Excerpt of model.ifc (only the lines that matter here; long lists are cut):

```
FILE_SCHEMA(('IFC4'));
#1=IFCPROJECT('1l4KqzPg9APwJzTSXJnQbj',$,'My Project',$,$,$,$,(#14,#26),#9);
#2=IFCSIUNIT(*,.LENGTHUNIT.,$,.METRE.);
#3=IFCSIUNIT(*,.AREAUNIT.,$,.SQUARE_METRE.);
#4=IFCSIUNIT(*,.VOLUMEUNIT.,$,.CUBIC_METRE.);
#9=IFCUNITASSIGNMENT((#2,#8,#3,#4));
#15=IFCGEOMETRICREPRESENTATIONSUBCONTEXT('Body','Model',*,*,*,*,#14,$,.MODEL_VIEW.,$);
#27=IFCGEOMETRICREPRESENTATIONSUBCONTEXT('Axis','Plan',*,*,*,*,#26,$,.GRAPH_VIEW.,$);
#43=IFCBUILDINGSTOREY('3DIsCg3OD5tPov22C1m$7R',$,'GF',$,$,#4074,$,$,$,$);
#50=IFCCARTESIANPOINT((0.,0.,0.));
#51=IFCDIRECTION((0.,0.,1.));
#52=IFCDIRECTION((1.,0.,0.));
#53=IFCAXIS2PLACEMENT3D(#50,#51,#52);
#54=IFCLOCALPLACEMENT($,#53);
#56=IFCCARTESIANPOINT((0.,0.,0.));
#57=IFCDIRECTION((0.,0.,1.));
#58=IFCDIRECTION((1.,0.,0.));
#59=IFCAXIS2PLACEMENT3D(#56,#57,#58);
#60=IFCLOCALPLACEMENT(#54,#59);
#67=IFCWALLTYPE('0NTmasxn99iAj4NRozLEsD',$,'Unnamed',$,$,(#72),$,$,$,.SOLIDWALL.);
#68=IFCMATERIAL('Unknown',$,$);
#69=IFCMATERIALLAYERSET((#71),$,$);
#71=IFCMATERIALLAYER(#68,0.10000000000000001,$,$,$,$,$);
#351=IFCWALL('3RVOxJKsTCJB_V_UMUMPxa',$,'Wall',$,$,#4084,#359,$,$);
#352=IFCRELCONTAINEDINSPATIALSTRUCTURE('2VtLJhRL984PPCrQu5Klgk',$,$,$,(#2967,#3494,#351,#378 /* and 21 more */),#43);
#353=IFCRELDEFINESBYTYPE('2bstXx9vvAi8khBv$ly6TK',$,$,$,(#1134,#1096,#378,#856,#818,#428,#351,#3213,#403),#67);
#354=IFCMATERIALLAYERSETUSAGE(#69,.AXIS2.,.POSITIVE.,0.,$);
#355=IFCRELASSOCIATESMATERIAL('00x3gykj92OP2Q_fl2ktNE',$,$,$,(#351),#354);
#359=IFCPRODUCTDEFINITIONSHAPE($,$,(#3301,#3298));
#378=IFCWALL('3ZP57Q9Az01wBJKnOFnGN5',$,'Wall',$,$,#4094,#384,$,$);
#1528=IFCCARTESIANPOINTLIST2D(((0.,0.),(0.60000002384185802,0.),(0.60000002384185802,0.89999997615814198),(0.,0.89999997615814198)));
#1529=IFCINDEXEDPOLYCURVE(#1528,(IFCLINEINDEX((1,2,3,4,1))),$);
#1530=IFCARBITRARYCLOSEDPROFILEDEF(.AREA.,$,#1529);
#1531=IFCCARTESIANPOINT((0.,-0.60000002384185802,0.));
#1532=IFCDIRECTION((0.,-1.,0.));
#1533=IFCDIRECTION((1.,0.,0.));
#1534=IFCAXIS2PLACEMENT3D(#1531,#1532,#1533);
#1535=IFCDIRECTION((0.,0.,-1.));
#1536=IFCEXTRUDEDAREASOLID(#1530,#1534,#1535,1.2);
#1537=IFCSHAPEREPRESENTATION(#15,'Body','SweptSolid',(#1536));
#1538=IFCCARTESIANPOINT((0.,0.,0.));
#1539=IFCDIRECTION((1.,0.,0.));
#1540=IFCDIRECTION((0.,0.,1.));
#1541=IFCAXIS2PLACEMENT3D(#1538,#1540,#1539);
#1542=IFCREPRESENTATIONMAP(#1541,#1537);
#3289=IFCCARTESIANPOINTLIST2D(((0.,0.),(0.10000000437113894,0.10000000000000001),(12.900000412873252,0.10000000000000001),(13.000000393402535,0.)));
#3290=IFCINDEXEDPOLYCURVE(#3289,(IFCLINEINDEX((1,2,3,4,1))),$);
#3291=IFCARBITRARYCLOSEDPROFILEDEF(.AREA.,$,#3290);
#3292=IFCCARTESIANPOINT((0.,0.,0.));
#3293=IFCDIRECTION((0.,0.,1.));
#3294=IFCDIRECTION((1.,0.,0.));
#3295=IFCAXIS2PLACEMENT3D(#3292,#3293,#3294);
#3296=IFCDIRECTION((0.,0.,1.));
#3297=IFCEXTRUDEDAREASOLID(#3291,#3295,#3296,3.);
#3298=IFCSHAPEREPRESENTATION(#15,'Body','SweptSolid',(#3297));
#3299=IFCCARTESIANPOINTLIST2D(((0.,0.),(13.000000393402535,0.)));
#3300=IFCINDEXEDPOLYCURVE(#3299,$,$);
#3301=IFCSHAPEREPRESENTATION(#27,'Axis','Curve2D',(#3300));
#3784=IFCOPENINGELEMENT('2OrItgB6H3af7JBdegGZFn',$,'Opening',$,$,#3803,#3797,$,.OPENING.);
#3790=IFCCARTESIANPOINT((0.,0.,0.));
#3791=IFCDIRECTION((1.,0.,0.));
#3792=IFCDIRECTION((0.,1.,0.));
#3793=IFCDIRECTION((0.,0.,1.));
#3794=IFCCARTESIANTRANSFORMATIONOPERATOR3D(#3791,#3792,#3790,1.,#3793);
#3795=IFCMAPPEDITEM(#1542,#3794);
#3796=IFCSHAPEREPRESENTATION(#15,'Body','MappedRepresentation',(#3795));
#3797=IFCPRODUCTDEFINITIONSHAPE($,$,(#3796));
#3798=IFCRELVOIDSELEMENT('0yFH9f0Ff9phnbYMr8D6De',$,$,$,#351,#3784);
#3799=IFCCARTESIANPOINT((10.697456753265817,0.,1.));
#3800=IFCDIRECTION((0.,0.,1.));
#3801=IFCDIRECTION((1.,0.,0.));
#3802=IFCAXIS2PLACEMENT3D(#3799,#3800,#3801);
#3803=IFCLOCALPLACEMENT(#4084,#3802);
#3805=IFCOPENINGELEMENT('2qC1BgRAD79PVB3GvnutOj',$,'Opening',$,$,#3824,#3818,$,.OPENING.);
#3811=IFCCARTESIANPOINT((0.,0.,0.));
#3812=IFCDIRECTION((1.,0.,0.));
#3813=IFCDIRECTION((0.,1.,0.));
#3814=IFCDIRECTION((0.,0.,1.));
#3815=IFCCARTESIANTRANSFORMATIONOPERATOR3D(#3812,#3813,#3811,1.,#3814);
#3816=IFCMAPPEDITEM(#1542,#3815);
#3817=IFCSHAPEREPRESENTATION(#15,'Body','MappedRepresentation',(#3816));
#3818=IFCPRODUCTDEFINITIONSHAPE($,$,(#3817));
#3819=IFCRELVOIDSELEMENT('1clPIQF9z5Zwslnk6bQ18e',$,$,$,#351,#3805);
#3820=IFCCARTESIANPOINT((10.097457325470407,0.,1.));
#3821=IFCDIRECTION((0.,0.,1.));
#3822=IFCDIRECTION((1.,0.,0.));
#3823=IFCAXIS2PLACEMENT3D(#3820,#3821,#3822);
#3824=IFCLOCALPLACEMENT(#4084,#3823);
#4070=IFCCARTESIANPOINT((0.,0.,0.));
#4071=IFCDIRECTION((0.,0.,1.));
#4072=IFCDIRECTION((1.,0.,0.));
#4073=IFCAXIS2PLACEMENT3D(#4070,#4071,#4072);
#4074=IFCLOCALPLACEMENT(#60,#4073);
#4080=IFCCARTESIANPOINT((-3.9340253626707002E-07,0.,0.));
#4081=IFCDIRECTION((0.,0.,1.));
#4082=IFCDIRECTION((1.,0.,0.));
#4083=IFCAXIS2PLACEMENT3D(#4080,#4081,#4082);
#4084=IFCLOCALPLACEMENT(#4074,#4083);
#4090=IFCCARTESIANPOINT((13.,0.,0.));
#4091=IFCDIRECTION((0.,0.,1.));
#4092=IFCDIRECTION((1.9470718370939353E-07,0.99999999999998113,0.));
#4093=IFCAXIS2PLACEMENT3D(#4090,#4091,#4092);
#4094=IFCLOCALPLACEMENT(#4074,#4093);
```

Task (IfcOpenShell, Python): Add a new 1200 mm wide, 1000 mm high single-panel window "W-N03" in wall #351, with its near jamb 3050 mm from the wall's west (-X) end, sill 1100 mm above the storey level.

```python
import numpy as np
import ifcopenshell
import ifcopenshell.api.feature
import ifcopenshell.api.geometry
import ifcopenshell.api.root
import ifcopenshell.api.spatial
import ifcopenshell.geom
import ifcopenshell.util.element
import ifcopenshell.util.placement
import ifcopenshell.util.representation
import ifcopenshell.util.shape
import ifcopenshell.util.unit

model = ifcopenshell.open("model.ifc")
unit_scale = ifcopenshell.util.unit.calculate_unit_scale(model)
settings = ifcopenshell.geom.settings()


def volume(element):
    """Net volume in cubic metres, openings subtracted."""
    shape = ifcopenshell.geom.create_shape(settings, element)
    return ifcopenshell.util.shape.get_volume(shape.geometry)


wall = model.by_guid("3RVOxJKsTCJB_V_UMUMPxa")
storey = ifcopenshell.util.element.get_container(wall, ifc_class="IfcBuildingStorey")
context = ifcopenshell.util.representation.get_context(model, "Model", "Body", "MODEL_VIEW")
before = volume(wall)

width, height, from_end, sill = 1.2, 1, 3.05, 1.1  # metres

# The wall runs along its own X axis, and the end named is its -X end.
wall_shape = ifcopenshell.geom.create_shape(settings, wall)
x, y, z = ifcopenshell.util.shape.get_vertices(wall_shape.geometry).T
start = x.min() + from_end
face, thickness = float(y.min()), float(y.max() - y.min())
wall_matrix = ifcopenshell.util.placement.get_local_placement(wall.ObjectPlacement)
level = ifcopenshell.util.placement.get_local_placement(storey.ObjectPlacement)[2, 3]


def in_wall(x, y):
    """Placement at x, y metres in the wall's axes, at sill height."""
    matrix = wall_matrix.copy()
    matrix[:, 3] = wall_matrix @ np.array([x / unit_scale, y / unit_scale, 0.0, 1.0])
    matrix[2, 3] = level + sill / unit_scale
    return matrix


# Opening: a box that overshoots both wall faces by 50 mm.
opening = ifcopenshell.api.root.create_entity(model, ifc_class="IfcOpeningElement", predefined_type="OPENING")
box = ifcopenshell.api.geometry.add_wall_representation(
    model, context=context, length=width, height=height, thickness=thickness + 0.1
)
ifcopenshell.api.geometry.assign_representation(model, product=opening, representation=box)
ifcopenshell.api.geometry.edit_object_placement(model, product=opening, matrix=in_wall(start, face - 0.05), is_si=False)
ifcopenshell.api.feature.add_feature(model, feature=opening, element=wall)

window = ifcopenshell.api.root.create_entity(model, ifc_class="IfcWindow", name="W-N03", predefined_type="WINDOW")
window.OverallWidth, window.OverallHeight = width / unit_scale, height / unit_scale
window.PartitioningType = "SINGLE_PANEL"
body = ifcopenshell.api.geometry.add_window_representation(
    model,
    context=context,
    overall_width=window.OverallWidth,
    overall_height=window.OverallHeight,
    partition_type="SINGLE_PANEL",
)
ifcopenshell.api.geometry.assign_representation(model, product=window, representation=body)
ifcopenshell.api.spatial.assign_container(model, products=[window], relating_structure=storey)
ifcopenshell.api.feature.add_filling(model, opening=opening, element=window)

# Centre the window in the wall's thickness.
ifcopenshell.api.geometry.edit_object_placement(model, product=window, matrix=in_wall(start, face), is_si=False)
window_shape = ifcopenshell.geom.create_shape(settings, window)
depth = ifcopenshell.util.shape.get_vertices(window_shape.geometry)[:, 1]
offset = face + thickness / 2 - (depth.min() + depth.max()) / 2
ifcopenshell.api.geometry.edit_object_placement(model, product=window, matrix=in_wall(start, offset), is_si=False)

after = volume(wall)

print(f"wall volume {before:.3f} -> {after:.3f} m3")

model.write("model_updated.ifc")
```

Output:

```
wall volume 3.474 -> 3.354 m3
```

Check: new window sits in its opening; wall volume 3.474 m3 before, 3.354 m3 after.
